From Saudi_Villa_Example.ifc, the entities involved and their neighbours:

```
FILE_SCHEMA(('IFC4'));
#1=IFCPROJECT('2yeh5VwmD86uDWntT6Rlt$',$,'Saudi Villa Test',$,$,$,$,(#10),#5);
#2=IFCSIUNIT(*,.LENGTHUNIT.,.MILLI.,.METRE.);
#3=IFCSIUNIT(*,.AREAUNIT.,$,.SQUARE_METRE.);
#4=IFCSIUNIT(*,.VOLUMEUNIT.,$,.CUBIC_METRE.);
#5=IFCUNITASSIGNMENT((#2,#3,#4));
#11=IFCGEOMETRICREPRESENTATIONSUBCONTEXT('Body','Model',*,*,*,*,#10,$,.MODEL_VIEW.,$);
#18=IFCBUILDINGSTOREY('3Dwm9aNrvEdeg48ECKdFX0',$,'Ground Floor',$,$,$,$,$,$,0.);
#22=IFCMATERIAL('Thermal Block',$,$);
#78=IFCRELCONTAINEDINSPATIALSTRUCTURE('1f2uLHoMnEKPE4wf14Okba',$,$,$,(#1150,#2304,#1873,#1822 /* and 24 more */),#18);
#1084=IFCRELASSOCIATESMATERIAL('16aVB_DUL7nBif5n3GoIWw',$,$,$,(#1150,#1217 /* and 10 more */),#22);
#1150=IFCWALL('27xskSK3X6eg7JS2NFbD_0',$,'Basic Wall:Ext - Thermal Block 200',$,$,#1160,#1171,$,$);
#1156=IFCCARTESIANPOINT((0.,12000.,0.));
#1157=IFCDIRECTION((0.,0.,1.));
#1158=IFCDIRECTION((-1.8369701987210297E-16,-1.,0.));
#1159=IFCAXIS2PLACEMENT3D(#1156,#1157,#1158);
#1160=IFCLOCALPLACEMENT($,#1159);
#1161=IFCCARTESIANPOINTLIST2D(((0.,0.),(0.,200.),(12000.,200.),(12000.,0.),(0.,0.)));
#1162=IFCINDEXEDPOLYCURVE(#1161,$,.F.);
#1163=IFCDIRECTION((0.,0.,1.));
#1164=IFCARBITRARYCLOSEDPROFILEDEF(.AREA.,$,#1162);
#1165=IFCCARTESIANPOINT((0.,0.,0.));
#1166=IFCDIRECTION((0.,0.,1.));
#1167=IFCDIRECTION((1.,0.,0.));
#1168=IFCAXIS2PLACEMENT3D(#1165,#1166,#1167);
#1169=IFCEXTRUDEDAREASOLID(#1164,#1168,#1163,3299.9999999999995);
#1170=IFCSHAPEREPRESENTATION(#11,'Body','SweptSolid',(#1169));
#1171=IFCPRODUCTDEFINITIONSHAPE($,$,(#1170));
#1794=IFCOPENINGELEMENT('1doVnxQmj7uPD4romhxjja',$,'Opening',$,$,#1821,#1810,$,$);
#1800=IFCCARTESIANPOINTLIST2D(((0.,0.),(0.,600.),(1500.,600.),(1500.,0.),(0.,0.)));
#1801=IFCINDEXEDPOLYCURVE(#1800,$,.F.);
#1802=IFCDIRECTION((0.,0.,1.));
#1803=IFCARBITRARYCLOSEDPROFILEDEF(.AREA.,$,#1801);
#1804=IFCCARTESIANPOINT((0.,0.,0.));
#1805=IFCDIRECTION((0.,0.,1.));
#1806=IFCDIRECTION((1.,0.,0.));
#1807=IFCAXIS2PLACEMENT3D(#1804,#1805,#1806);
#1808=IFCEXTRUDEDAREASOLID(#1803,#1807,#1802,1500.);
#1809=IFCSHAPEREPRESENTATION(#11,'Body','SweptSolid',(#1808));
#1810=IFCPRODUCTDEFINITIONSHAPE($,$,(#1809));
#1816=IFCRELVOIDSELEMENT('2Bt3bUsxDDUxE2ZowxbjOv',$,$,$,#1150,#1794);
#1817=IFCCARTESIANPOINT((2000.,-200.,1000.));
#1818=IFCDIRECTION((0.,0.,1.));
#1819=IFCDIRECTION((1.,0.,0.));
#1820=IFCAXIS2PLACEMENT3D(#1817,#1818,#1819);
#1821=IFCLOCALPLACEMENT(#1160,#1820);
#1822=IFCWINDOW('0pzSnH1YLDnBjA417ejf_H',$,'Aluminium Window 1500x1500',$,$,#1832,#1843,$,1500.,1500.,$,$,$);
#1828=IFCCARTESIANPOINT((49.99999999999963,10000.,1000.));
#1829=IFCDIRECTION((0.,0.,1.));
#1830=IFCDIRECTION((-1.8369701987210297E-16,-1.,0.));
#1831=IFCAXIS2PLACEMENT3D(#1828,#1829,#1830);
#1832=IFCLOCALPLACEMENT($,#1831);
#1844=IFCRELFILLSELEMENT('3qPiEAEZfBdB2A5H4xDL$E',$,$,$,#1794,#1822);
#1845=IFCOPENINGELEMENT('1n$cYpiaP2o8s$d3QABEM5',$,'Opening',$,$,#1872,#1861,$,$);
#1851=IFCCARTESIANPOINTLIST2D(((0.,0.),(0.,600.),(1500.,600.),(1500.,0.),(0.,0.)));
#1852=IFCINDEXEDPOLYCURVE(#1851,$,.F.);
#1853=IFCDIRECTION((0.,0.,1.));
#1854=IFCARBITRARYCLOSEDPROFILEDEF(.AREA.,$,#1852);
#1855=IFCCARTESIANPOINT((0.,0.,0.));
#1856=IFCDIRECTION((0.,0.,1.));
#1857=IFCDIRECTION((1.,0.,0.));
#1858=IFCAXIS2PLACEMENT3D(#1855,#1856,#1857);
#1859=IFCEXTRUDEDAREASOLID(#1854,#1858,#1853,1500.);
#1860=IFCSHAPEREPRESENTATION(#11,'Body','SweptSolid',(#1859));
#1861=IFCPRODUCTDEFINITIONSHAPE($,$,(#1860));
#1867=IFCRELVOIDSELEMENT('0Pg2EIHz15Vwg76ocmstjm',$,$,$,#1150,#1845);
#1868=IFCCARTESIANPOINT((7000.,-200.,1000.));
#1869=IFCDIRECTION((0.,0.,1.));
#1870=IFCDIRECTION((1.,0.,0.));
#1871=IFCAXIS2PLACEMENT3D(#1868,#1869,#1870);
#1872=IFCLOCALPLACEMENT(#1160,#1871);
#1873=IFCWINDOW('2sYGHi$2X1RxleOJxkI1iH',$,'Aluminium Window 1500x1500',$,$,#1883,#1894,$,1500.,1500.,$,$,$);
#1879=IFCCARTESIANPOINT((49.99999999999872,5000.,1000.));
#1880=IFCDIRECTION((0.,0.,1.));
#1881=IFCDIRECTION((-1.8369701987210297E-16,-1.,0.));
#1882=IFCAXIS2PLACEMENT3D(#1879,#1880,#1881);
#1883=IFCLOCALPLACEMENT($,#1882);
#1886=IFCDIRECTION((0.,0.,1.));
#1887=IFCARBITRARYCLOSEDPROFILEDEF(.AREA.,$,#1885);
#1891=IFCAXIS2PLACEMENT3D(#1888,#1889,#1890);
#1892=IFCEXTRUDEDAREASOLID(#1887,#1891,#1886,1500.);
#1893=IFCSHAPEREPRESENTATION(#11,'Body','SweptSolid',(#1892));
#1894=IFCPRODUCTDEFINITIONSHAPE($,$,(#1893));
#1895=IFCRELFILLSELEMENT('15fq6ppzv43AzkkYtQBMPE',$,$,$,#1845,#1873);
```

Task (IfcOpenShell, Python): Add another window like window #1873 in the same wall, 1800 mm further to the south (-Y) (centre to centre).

```python
import ifcopenshell
import ifcopenshell.api.feature
import ifcopenshell.api.geometry
import ifcopenshell.api.root
import ifcopenshell.geom
import ifcopenshell.util.element
import ifcopenshell.util.placement
import ifcopenshell.util.shape
import ifcopenshell.util.unit

model = ifcopenshell.open("Saudi_Villa_Example.ifc")
unit_scale = ifcopenshell.util.unit.calculate_unit_scale(model)
settings = ifcopenshell.geom.settings()


def volume(element):
    """Net volume in cubic metres, openings subtracted."""
    shape = ifcopenshell.geom.create_shape(settings, element)
    return ifcopenshell.util.shape.get_volume(shape.geometry)


window = model.by_guid("2sYGHi$2X1RxleOJxkI1iH")
opening = window.FillsVoids[0].RelatingOpeningElement
wall = opening.VoidsElements[0].RelatingBuildingElement
before = volume(wall)
shift = ifcopenshell.util.placement.get_local_placement(wall.ObjectPlacement)[:3, 0] * 1.8 / unit_scale

# copy_class copies the void relationship, type, container and properties, but no geometry.
new_opening = ifcopenshell.api.root.copy_class(model, product=opening)
new_opening.Representation = ifcopenshell.util.element.copy_deep(
    model, opening.Representation, exclude=["IfcGeometricRepresentationContext", "IfcRepresentationMap"]
)
new_window = ifcopenshell.api.root.copy_class(model, product=window)
new_window.Representation = ifcopenshell.util.element.copy_deep(
    model, window.Representation, exclude=["IfcGeometricRepresentationContext", "IfcRepresentationMap"]
)
ifcopenshell.api.feature.add_filling(model, opening=new_opening, element=new_window)

for old, new in ((opening, new_opening), (window, new_window)):
    matrix = ifcopenshell.util.placement.get_local_placement(old.ObjectPlacement)
    matrix[:3, 3] += shift
    ifcopenshell.api.geometry.edit_object_placement(model, product=new, matrix=matrix, is_si=False)

after = volume(wall)

print(f"wall volume {before:.3f} -> {after:.3f} m3")

model.write("Saudi_Villa_Example_edited.ifc")
```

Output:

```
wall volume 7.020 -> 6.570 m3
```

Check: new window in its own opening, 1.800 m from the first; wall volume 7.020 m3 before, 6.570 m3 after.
